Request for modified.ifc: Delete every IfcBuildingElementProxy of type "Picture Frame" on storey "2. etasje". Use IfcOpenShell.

First a look at what the model holds.

```python
import ifcopenshell
import ifcopenshell.util.element

model = ifcopenshell.open("modified.ifc")
print(model.schema)
storey = next(s for s in model.by_type("IfcBuildingStorey") if s.Name == "2. etasje")
proxies = [e for e in ifcopenshell.util.element.get_decomposition(storey) if e.is_a("IfcBuildingElementProxy")]
seen = {}
for e in proxies:
    element_type = ifcopenshell.util.element.get_type(e)
    name = element_type.Name if element_type not in (None, e) else None
    seen[name] = seen.get(name, 0) + 1
for name, count in sorted(seen.items(), key=str):
    print(count, "x", name)
```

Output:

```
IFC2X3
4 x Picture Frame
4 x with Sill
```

```python
import ifcopenshell
import ifcopenshell.api.root
import ifcopenshell.util.element

model = ifcopenshell.open("modified.ifc")

storey = next(s for s in model.by_type("IfcBuildingStorey") if s.Name == "2. etasje")
proxies = [e for e in ifcopenshell.util.element.get_decomposition(storey) if e.is_a("IfcBuildingElementProxy")]
targets = [e for e in proxies if (t := ifcopenshell.util.element.get_type(e)) not in (None, e) and t.Name == "Picture Frame"]

for e in targets:
    ifcopenshell.api.root.remove_product(model, product=e)
print(len(targets), "removed")

model.write("modified_v2.ifc")
```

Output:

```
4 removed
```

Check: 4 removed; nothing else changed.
